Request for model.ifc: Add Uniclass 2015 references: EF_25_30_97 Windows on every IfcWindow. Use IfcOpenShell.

First a look at what the model holds.

```python
import ifcopenshell

model = ifcopenshell.open("model.ifc")
print(model.schema)
print("classifications:", [c.Name for c in model.by_type("IfcClassification")])
for ifc_class in ("IfcDoor", "IfcRoof", "IfcStair", "IfcWall", "IfcWindow"):
    print(ifc_class, len(model.by_type(ifc_class)))
```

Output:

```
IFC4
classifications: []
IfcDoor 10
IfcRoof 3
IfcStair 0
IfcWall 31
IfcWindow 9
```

```python
import ifcopenshell
import ifcopenshell.api.classification

model = ifcopenshell.open("model.ifc")

system = ifcopenshell.api.classification.add_classification(model, classification="Uniclass 2015")

codes = {
    "IfcWindow": ("EF_25_30_97", "Windows"),
}
for ifc_class, (code, name) in codes.items():
    products = model.by_type(ifc_class)
    ifcopenshell.api.classification.add_reference(
        model, products=products, classification=system, identification=code, name=name
    )
    print(code, len(products))

model.write("model-out.ifc")
```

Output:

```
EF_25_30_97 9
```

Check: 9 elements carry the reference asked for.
